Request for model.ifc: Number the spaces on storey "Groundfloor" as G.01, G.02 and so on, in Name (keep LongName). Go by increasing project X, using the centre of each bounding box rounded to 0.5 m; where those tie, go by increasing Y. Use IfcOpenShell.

First a look at what the model holds.

```python
import ifcopenshell
import ifcopenshell.util.element
import ifcopenshell.util.placement

model = ifcopenshell.open("model.ifc")
print(model.schema)
storey = next(s for s in model.by_type("IfcBuildingStorey") if s.Name == "Groundfloor")
spaces = [e for e in ifcopenshell.util.element.get_decomposition(storey) if e.is_a("IfcSpace")]
for e in sorted(spaces, key=lambda e: e.id()):
    origin = ifcopenshell.util.placement.get_local_placement(e.ObjectPlacement)[:3, 3]
    print(e.id(), e.Name, e.LongName, origin.round(2) + 0.0, sep=" | ")
```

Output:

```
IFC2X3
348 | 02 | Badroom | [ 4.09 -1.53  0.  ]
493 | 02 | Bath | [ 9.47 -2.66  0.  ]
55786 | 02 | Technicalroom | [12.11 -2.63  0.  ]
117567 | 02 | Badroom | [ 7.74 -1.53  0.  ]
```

```python
import ifcopenshell
import ifcopenshell.geom
import ifcopenshell.util.element
import ifcopenshell.util.shape

model = ifcopenshell.open("model.ifc")
settings = ifcopenshell.geom.settings()
settings.set("use-world-coords", True)


def centre(element):
    shape = ifcopenshell.geom.create_shape(settings, element)
    return ifcopenshell.util.shape.get_bbox_centroid(shape.geometry)


storey = next(s for s in model.by_type("IfcBuildingStorey") if s.Name == "Groundfloor")
spaces = [e for e in ifcopenshell.util.element.get_decomposition(storey) if e.is_a("IfcSpace")]

# Insertion points can sit at a corner or the storey origin, so sort by the geometry (in metres).
centres = {e: centre(e) for e in spaces}
spaces.sort(key=lambda e: (round(centres[e][0] / 0.5), centres[e][1]))

for i, e in enumerate(spaces, start=1):
    number = f"G.{i:02d}"
    e.Name = number
    print(e.id(), number)

model.write("model_rev.ifc")
```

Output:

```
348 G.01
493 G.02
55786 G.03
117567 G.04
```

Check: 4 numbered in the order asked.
